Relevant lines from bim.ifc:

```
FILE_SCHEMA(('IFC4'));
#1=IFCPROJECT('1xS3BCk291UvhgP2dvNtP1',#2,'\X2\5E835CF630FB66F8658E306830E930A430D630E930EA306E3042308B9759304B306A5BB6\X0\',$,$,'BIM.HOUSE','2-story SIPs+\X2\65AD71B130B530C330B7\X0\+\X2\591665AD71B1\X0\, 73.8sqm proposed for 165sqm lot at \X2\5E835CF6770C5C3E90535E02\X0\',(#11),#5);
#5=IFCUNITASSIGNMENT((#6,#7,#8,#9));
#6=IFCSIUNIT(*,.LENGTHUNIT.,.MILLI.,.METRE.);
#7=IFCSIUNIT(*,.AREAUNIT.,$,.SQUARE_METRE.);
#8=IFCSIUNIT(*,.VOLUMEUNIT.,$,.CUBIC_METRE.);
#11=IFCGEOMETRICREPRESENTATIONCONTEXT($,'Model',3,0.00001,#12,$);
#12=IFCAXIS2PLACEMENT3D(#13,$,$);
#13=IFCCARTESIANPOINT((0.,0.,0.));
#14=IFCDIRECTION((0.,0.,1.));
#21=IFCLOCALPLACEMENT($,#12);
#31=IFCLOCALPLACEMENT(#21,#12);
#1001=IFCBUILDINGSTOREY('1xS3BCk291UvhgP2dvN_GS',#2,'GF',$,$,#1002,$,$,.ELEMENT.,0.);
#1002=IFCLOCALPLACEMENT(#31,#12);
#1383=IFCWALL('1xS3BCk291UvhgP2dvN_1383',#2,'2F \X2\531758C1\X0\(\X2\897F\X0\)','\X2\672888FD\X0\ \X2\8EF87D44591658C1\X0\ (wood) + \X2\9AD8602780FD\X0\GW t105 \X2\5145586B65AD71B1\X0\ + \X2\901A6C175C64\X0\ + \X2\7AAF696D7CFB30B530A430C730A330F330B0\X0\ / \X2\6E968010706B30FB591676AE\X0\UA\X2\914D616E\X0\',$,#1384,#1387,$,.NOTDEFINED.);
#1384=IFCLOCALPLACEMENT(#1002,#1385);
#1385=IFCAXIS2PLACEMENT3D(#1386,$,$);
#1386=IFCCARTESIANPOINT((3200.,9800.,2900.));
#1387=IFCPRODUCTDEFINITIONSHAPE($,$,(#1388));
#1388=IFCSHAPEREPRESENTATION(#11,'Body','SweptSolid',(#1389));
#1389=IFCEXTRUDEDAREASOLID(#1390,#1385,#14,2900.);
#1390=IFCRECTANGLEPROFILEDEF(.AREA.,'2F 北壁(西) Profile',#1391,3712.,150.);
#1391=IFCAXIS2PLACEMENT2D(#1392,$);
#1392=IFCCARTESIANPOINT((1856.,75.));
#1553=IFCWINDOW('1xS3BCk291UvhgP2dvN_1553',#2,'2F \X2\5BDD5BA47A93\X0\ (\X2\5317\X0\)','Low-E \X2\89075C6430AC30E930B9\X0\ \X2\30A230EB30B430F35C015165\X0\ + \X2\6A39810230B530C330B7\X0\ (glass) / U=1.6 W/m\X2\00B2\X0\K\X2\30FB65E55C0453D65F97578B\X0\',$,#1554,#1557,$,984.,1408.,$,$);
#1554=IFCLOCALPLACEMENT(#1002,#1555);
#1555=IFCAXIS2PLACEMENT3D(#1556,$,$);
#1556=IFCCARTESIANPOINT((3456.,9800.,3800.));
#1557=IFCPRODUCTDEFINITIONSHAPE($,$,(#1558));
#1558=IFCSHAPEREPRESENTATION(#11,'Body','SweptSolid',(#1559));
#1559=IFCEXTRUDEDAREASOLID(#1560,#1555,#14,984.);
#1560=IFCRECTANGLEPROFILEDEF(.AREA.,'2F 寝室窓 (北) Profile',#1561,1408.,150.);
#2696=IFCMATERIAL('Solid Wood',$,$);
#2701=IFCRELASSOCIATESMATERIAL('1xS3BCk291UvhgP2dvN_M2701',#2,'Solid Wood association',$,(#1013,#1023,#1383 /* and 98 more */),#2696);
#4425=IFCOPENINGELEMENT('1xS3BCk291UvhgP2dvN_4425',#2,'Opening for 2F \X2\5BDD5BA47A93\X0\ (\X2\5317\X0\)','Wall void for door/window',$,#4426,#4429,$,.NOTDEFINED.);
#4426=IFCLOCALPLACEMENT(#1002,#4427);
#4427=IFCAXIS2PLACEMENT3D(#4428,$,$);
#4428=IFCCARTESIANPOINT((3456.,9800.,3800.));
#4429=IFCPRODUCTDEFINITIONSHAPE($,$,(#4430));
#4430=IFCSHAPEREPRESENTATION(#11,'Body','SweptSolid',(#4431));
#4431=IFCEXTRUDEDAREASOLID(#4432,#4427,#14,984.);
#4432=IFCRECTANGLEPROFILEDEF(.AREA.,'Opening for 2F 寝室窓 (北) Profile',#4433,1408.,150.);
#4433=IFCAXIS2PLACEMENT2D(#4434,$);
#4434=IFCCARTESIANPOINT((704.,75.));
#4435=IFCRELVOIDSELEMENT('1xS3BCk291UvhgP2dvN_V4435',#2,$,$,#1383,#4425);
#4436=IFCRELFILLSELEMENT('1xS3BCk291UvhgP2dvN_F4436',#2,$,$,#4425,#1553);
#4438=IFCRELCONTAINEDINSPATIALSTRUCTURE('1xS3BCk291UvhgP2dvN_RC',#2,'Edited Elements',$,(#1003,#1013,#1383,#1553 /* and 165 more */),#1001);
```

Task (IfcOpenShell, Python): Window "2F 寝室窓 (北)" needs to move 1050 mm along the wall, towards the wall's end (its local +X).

```python
import ifcopenshell
import ifcopenshell.api.geometry
import ifcopenshell.util.placement
import ifcopenshell.util.unit

model = ifcopenshell.open("bim.ifc")
unit_scale = ifcopenshell.util.unit.calculate_unit_scale(model)

window = model.by_guid("1xS3BCk291UvhgP2dvN_1553")
opening = window.FillsVoids[0].RelatingOpeningElement
wall = opening.VoidsElements[0].RelatingBuildingElement

wall_matrix = ifcopenshell.util.placement.get_local_placement(wall.ObjectPlacement)
shift = wall_matrix[:3, 0] * 1.05 / unit_scale
before = ifcopenshell.util.placement.get_local_placement(window.ObjectPlacement)[:3, 3].copy()

# The window is not placed relative to its opening, so move both.
for product in (opening, window):
    matrix = ifcopenshell.util.placement.get_local_placement(product.ObjectPlacement)
    matrix[:3, 3] += shift
    ifcopenshell.api.geometry.edit_object_placement(model, product=product, matrix=matrix, is_si=False)

after = ifcopenshell.util.placement.get_local_placement(window.ObjectPlacement)[:3, 3]
print("window moved by", (after - before).round(3) + 0.0)

model.write("bim_v2.ifc")
```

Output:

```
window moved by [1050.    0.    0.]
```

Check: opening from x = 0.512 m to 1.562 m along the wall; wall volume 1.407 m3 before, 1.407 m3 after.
